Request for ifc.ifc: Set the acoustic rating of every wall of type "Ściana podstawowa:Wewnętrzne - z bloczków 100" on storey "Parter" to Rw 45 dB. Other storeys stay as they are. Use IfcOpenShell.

First a look at what the model holds.

```python
import ifcopenshell
import ifcopenshell.util.element

model = ifcopenshell.open("ifc.ifc")
print(model.schema)
storey = next(s for s in model.by_type("IfcBuildingStorey") if s.Name == "Parter")
walls = [e for e in ifcopenshell.util.element.get_decomposition(storey) if e.is_a("IfcWall")]
seen = {}
for e in walls:
    element_type = ifcopenshell.util.element.get_type(e)
    key = (element_type.Name if element_type != e and element_type else None, ifcopenshell.util.element.get_pset(e, "Pset_WallCommon", "AcousticRating"))
    seen[key] = seen.get(key, 0) + 1
for (name, value), count in sorted(seen.items(), key=str):
    print(count, "x", name, "|", value)
```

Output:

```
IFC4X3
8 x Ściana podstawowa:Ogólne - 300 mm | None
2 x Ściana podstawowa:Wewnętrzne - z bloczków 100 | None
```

```python
import ifcopenshell
import ifcopenshell.api.pset
import ifcopenshell.util.element

model = ifcopenshell.open("ifc.ifc")

storey = next(s for s in model.by_type("IfcBuildingStorey") if s.Name == "Parter")
walls = [e for e in ifcopenshell.util.element.get_decomposition(storey) if e.is_a("IfcWall")]

count = 0
for e in walls:
    element_type = ifcopenshell.util.element.get_type(e)
    if element_type in (None, e) or element_type.Name != "Ściana podstawowa:Wewnętrzne - z bloczków 100":
        continue
    # add_pset returns the element's existing set when there is one.
    pset = ifcopenshell.api.pset.add_pset(model, product=e, name="Pset_WallCommon")
    ifcopenshell.api.pset.edit_pset(model, pset=pset, properties={"AcousticRating": "Rw 45 dB"})
    count += 1

print(count, "walls updated")

model.write("ifc_updated.ifc")
```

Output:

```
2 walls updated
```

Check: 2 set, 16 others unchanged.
